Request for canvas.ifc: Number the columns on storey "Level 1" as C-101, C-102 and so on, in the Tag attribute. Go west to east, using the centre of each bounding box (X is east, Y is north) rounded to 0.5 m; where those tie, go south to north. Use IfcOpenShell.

First a look at what the model holds.

```python
import ifcopenshell
import ifcopenshell.util.element
import ifcopenshell.util.placement

model = ifcopenshell.open("canvas.ifc")
print(model.schema)
storey = next(s for s in model.by_type("IfcBuildingStorey") if s.Name == "Level 1")
columns = [e for e in ifcopenshell.util.element.get_decomposition(storey) if e.is_a("IfcColumn")]
for e in sorted(columns, key=lambda e: e.id()):
    origin = ifcopenshell.util.placement.get_local_placement(e.ObjectPlacement)[:3, 3]
    print(e.id(), e.Tag, e.Name, origin.round(2) + 0.0, sep=" | ")
```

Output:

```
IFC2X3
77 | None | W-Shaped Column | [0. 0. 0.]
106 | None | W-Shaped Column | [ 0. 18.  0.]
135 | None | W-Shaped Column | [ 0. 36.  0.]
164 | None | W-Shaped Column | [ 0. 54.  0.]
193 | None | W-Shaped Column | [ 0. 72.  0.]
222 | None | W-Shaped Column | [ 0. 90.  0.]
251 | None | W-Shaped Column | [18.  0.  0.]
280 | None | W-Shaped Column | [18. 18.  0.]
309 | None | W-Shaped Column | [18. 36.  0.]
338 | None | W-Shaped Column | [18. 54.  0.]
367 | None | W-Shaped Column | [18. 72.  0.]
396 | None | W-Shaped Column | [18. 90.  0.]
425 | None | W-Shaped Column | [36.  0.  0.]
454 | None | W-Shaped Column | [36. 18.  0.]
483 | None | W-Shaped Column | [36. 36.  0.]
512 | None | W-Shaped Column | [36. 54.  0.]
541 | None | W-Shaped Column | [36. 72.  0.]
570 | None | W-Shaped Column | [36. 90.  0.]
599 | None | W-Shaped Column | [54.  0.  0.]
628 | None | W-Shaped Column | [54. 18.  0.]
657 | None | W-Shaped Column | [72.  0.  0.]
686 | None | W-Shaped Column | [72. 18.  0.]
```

```python
import ifcopenshell
import ifcopenshell.geom
import ifcopenshell.util.element
import ifcopenshell.util.shape

model = ifcopenshell.open("canvas.ifc")
settings = ifcopenshell.geom.settings()
settings.set("use-world-coords", True)


def centre(element):
    shape = ifcopenshell.geom.create_shape(settings, element)
    return ifcopenshell.util.shape.get_bbox_centroid(shape.geometry)


storey = next(s for s in model.by_type("IfcBuildingStorey") if s.Name == "Level 1")
columns = [e for e in ifcopenshell.util.element.get_decomposition(storey) if e.is_a("IfcColumn")]

# Insertion points can sit at a corner or the storey origin, so sort by the geometry (in metres).
centres = {e: centre(e) for e in columns}
columns.sort(key=lambda e: (round(centres[e][0] / 0.5), centres[e][1]))

for i, e in enumerate(columns, start=1):
    number = f"C-1{i:02d}"
    e.Tag = number
    print(e.id(), number)

model.write("canvas_edited.ifc")
```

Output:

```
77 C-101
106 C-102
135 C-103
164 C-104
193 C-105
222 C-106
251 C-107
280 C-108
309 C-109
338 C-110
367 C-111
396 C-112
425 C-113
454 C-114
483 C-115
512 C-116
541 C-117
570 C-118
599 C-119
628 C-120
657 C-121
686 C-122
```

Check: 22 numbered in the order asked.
